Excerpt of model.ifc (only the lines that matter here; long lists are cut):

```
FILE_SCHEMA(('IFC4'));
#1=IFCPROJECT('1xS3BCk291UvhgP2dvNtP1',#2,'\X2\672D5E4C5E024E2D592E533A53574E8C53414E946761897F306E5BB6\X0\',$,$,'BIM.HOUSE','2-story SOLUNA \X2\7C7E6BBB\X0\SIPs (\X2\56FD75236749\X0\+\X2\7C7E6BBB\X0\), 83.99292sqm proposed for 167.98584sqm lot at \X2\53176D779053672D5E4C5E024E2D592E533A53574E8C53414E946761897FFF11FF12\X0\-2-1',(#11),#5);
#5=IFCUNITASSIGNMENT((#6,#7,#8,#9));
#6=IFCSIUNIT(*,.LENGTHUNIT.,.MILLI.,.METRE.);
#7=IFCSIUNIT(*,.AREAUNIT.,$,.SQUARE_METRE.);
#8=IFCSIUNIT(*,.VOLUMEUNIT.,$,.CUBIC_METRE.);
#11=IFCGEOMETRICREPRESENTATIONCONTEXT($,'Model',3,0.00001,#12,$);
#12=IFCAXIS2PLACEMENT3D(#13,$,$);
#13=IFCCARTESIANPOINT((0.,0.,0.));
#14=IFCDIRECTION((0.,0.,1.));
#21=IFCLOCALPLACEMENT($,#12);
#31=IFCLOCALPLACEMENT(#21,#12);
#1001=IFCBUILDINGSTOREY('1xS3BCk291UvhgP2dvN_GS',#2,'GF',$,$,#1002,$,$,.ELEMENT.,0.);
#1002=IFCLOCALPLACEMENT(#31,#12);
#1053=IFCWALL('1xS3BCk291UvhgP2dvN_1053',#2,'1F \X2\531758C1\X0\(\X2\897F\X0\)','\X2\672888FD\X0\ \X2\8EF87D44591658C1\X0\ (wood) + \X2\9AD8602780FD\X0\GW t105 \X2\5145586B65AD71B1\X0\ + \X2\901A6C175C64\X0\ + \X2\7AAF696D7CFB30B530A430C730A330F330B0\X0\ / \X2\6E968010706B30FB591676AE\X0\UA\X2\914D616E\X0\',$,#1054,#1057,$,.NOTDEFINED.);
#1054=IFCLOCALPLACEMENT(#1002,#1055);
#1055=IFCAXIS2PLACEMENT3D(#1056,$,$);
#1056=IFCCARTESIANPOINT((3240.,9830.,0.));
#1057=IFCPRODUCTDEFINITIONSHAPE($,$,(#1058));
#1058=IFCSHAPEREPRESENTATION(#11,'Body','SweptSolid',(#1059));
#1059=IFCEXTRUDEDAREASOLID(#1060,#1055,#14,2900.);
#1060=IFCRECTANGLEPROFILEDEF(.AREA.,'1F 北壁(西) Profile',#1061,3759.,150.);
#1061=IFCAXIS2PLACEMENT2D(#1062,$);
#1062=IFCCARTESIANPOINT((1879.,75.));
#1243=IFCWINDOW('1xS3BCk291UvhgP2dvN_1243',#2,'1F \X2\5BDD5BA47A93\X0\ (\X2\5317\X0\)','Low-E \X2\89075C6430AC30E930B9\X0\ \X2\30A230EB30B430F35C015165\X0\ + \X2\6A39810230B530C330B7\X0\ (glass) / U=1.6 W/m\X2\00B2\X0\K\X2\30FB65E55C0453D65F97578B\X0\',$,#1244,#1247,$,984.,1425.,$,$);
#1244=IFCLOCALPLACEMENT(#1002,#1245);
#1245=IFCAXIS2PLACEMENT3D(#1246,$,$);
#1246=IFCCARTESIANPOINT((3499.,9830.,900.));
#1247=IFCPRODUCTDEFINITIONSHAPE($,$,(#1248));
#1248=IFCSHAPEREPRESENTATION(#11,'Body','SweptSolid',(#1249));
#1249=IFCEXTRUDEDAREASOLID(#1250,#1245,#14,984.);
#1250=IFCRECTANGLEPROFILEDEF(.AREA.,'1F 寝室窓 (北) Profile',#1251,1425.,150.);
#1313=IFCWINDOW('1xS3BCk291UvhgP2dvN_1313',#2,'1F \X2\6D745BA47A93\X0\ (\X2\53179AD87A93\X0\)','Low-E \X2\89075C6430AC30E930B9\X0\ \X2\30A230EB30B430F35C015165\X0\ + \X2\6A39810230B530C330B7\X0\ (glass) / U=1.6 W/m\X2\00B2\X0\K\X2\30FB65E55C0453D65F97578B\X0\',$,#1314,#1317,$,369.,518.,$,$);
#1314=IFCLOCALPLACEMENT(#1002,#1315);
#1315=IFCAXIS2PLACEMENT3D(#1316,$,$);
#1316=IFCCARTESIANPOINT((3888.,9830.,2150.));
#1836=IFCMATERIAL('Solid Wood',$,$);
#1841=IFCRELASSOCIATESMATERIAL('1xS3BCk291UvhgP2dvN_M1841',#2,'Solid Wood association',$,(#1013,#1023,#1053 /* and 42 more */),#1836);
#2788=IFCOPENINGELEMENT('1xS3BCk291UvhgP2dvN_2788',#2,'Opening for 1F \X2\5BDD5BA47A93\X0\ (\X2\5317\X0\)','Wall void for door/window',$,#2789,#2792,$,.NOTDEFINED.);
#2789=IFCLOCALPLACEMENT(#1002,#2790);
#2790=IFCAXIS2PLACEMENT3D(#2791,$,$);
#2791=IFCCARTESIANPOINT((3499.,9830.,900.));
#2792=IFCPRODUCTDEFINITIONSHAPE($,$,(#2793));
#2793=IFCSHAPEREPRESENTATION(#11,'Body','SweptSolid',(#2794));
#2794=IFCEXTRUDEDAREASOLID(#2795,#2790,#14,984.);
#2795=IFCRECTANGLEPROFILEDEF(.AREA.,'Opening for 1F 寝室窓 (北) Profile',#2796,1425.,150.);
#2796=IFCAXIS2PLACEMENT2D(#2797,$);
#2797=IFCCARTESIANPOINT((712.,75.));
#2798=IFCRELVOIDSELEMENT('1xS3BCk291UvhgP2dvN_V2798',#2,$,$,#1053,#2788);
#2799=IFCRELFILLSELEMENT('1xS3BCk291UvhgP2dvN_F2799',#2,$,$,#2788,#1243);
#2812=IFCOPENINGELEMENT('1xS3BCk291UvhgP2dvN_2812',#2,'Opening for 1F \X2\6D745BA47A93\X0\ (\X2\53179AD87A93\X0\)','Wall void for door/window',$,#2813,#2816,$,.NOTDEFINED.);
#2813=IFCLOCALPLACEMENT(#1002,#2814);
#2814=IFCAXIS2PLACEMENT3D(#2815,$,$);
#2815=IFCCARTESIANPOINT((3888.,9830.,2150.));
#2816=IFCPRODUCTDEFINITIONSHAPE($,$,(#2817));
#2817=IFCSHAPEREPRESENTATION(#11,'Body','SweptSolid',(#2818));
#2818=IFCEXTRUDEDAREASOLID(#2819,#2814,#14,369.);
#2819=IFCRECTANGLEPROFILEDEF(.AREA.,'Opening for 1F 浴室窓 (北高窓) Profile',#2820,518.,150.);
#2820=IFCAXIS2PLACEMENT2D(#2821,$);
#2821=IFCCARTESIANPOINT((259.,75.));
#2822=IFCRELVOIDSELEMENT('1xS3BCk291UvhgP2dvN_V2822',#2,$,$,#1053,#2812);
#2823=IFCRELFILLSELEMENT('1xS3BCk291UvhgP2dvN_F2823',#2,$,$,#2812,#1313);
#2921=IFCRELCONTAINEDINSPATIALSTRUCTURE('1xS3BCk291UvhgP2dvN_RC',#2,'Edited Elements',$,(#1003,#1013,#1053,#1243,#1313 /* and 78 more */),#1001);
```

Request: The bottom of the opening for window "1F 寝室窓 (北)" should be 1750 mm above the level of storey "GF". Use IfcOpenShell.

```python
import numpy as np
import ifcopenshell
import ifcopenshell.api.geometry
import ifcopenshell.geom
import ifcopenshell.util.element
import ifcopenshell.util.placement
import ifcopenshell.util.shape
import ifcopenshell.util.unit

model = ifcopenshell.open("model.ifc")
unit_scale = ifcopenshell.util.unit.calculate_unit_scale(model)

window = model.by_guid("1xS3BCk291UvhgP2dvN_1243")
opening = window.FillsVoids[0].RelatingOpeningElement
storey = ifcopenshell.util.element.get_container(window, ifc_class="IfcBuildingStorey")
level = ifcopenshell.util.placement.get_local_placement(storey.ObjectPlacement)[2, 3]

# The opening's origin need not be at the sill, so measure its lowest point.
shape = ifcopenshell.geom.create_shape(ifcopenshell.geom.settings(), opening)
bottom = ifcopenshell.util.shape.get_shape_bottom_elevation(shape, shape.geometry) / unit_scale
dz = level + 1750.0 - bottom

shift = np.array([0.0, 0.0, dz])
# The window is not placed relative to its opening, so move both.
for product in (opening, window):
    matrix = ifcopenshell.util.placement.get_local_placement(product.ObjectPlacement)
    matrix[:3, 3] += shift
    ifcopenshell.api.geometry.edit_object_placement(model, product=product, matrix=matrix, is_si=False)

print(f"moved by {dz * unit_scale:+.3f} m")

model.write("model-out.ifc")
```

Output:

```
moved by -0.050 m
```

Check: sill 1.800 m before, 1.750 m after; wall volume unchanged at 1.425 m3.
